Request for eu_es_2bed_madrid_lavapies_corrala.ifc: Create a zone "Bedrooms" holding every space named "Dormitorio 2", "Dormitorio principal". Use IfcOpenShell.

First a look at what the model holds.

```python
import ifcopenshell

model = ifcopenshell.open("eu_es_2bed_madrid_lavapies_corrala.ifc")
print(model.schema)
seen = {}
for space in model.by_type("IfcSpace"):
    seen[space.LongName] = seen.get(space.LongName, 0) + 1
for name, count in sorted(seen.items(), key=str):
    print(count, "x", name)
print("zones:", [z.Name for z in model.by_type("IfcZone")][:20])
```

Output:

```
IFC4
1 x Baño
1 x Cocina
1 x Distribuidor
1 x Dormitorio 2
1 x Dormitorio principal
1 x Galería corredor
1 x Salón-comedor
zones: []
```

```python
import ifcopenshell
import ifcopenshell.api.group
import ifcopenshell.api.root

model = ifcopenshell.open("eu_es_2bed_madrid_lavapies_corrala.ifc")

names = {"Dormitorio 2", "Dormitorio principal"}
spaces = [s for s in model.by_type("IfcSpace") if s.LongName in names]

zone = ifcopenshell.api.root.create_entity(model, ifc_class="IfcZone", name="Bedrooms")
ifcopenshell.api.group.assign_group(model, products=spaces, group=zone)
print(len(spaces), "spaces in", zone.Name)

model.write("eu_es_2bed_madrid_lavapies_corrala_edited.ifc")
```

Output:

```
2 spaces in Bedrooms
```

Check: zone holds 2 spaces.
